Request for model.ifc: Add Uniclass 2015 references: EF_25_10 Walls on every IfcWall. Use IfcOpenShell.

First a look at what the model holds.

```python
import ifcopenshell

model = ifcopenshell.open("model.ifc")
print(model.schema)
print("classifications:", [c.Name for c in model.by_type("IfcClassification")])
for ifc_class in ("IfcDoor", "IfcRoof", "IfcStair", "IfcWall", "IfcWindow"):
    print(ifc_class, len(model.by_type(ifc_class)))
```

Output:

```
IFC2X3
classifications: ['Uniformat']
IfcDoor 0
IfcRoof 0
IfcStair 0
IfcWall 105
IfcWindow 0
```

```python
import ifcopenshell
import ifcopenshell.api.classification

model = ifcopenshell.open("model.ifc")

# IFC2X3 requires Source and Edition and has no link from the project to the system.
system = model.create_entity("IfcClassification", Source="NBS", Edition="2015", Name="Uniclass 2015")

codes = {
    "IfcWall": ("EF_25_10", "Walls"),
}
for ifc_class, (code, name) in codes.items():
    products = model.by_type(ifc_class)
    ifcopenshell.api.classification.add_reference(
        model, products=products, classification=system, identification=code, name=name
    )
    print(code, len(products))

model.write("model_v2.ifc")
```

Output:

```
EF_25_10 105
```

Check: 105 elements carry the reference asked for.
